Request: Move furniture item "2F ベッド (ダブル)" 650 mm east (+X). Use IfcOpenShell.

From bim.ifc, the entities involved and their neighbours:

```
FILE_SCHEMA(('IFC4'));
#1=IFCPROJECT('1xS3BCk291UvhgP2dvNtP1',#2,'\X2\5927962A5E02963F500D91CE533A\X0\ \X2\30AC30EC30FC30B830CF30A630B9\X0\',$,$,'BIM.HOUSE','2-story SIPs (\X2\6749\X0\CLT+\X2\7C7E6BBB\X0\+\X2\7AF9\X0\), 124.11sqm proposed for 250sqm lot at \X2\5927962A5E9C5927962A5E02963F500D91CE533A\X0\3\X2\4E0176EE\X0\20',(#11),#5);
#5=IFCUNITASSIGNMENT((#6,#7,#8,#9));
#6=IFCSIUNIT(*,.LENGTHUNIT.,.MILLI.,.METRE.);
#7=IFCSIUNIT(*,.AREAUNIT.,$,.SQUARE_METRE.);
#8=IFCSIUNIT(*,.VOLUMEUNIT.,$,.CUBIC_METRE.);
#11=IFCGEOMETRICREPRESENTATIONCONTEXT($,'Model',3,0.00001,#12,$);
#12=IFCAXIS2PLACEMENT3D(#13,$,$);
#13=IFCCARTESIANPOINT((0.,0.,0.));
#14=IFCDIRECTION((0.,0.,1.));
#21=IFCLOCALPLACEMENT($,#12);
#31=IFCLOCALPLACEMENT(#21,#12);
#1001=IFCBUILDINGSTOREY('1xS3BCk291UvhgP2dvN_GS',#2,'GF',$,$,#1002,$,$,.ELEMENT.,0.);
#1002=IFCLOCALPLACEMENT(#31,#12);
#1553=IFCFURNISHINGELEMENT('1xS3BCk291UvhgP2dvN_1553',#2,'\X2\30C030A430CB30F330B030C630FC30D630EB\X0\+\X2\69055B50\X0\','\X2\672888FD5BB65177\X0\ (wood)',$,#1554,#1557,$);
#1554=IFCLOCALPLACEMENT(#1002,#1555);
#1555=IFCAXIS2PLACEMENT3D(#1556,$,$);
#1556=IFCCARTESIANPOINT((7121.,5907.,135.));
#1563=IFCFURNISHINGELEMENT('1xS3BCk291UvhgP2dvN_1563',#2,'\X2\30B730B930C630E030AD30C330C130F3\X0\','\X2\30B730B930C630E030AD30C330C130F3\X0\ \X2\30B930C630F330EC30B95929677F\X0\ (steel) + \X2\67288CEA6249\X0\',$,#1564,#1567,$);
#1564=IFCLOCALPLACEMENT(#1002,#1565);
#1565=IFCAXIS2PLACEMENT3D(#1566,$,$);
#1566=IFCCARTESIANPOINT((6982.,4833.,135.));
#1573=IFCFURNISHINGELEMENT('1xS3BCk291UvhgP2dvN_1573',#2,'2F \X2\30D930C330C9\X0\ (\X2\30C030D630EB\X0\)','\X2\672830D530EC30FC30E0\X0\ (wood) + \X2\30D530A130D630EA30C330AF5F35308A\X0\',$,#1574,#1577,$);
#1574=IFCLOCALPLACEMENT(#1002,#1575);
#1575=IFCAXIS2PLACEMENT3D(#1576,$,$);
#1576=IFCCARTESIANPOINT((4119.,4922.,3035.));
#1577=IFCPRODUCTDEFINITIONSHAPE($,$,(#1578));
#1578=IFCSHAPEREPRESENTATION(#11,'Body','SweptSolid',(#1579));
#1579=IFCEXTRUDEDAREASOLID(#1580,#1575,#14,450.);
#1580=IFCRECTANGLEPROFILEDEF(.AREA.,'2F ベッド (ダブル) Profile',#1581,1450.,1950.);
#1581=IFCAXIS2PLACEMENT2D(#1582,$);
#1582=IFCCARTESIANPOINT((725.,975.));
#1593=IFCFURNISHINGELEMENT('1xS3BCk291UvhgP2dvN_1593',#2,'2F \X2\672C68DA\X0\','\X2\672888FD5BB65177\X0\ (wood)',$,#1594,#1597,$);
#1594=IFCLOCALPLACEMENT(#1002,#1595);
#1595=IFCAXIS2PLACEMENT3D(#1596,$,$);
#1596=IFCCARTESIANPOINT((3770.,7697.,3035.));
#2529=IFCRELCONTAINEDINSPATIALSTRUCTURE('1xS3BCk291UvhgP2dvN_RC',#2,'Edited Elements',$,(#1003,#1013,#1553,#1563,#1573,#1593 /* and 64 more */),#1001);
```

```python
import ifcopenshell
import ifcopenshell.api.geometry
import ifcopenshell.util.placement
import ifcopenshell.util.unit

model = ifcopenshell.open("bim.ifc")
unit_scale = ifcopenshell.util.unit.calculate_unit_scale(model)

item = model.by_id(1573)
matrix = ifcopenshell.util.placement.get_local_placement(item.ObjectPlacement)
matrix[0, 3] += 0.65 / unit_scale
ifcopenshell.api.geometry.edit_object_placement(model, product=item, matrix=matrix, is_si=False)

print(ifcopenshell.util.placement.get_local_placement(item.ObjectPlacement).round(3) + 0.0)

model.write("bim_v2.ifc")
```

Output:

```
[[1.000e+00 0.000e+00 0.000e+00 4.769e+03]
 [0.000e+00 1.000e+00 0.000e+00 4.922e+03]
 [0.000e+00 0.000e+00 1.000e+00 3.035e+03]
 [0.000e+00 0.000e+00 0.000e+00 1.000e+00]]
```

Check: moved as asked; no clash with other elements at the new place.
